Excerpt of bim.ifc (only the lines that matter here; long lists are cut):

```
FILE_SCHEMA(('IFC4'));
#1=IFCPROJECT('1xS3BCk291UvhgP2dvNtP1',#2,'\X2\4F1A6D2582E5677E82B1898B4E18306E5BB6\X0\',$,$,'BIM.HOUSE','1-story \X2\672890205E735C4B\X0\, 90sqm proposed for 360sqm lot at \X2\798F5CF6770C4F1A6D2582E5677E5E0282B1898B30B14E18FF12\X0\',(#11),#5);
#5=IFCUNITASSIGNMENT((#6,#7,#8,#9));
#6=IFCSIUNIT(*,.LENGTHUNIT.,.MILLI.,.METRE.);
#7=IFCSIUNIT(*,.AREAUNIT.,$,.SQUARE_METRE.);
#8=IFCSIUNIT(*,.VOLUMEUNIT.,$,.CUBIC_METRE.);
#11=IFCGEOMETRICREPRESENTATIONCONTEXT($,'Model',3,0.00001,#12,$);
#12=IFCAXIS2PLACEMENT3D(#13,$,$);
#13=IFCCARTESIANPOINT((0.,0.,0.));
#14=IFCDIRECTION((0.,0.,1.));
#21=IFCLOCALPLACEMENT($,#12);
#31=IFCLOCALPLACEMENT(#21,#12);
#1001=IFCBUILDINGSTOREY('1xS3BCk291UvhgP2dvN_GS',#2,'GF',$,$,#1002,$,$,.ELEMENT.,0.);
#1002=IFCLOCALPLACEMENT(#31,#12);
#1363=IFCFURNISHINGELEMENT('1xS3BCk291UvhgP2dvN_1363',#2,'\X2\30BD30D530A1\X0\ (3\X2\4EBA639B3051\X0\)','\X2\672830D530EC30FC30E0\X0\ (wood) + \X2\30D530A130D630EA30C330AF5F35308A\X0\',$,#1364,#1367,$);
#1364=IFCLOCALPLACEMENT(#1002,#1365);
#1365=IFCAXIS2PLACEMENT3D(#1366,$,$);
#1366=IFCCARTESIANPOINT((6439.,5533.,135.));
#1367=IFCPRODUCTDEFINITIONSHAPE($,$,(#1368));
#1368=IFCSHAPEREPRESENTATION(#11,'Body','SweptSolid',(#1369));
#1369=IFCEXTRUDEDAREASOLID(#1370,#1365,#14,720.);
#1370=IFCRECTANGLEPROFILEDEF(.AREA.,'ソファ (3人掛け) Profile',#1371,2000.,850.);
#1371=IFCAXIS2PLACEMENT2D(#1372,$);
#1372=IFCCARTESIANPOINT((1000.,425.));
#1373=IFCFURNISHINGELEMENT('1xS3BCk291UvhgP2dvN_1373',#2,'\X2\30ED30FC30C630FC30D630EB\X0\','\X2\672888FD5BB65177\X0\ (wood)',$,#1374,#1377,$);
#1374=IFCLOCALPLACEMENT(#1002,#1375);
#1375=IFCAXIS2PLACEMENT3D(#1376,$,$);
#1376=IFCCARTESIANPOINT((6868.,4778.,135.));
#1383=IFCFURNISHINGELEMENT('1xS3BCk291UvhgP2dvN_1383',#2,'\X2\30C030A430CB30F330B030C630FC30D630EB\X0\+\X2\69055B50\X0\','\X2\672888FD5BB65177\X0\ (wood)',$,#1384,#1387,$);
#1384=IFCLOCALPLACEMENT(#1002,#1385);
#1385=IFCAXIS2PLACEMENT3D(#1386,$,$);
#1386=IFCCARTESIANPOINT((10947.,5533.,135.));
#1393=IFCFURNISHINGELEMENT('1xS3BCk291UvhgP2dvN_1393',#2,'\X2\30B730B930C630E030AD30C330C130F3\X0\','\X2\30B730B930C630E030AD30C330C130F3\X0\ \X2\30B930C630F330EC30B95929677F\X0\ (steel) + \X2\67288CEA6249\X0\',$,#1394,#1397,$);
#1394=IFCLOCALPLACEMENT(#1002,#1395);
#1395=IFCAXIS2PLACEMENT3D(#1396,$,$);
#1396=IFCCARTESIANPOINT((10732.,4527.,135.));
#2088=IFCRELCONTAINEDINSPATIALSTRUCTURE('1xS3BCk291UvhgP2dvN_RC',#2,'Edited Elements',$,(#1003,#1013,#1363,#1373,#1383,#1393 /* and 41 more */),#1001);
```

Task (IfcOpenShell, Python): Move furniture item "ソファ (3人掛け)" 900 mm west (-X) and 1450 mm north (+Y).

```python
import ifcopenshell
import ifcopenshell.api.geometry
import ifcopenshell.util.placement
import ifcopenshell.util.unit

model = ifcopenshell.open("bim.ifc")
unit_scale = ifcopenshell.util.unit.calculate_unit_scale(model)

item = model.by_id(1363)
matrix = ifcopenshell.util.placement.get_local_placement(item.ObjectPlacement)
matrix[0, 3] -= 0.9 / unit_scale
matrix[1, 3] += 1.45 / unit_scale
ifcopenshell.api.geometry.edit_object_placement(model, product=item, matrix=matrix, is_si=False)

print(ifcopenshell.util.placement.get_local_placement(item.ObjectPlacement).round(3) + 0.0)

model.write("bim_edited.ifc")
```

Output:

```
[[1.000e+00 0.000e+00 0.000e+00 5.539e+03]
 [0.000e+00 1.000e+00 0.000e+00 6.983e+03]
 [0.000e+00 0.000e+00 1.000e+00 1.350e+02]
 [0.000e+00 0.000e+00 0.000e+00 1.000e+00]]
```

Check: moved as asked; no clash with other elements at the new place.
